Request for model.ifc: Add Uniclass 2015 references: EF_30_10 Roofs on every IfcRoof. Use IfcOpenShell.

First a look at what the model holds.

```python
import ifcopenshell

model = ifcopenshell.open("model.ifc")
print(model.schema)
print("classifications:", [c.Name for c in model.by_type("IfcClassification")])
for ifc_class in ("IfcDoor", "IfcRoof", "IfcStair", "IfcWall", "IfcWindow"):
    print(ifc_class, len(model.by_type(ifc_class)))
```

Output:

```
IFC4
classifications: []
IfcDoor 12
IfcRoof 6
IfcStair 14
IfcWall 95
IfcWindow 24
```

```python
import ifcopenshell
import ifcopenshell.api.classification

model = ifcopenshell.open("model.ifc")

system = ifcopenshell.api.classification.add_classification(model, classification="Uniclass 2015")

codes = {
    "IfcRoof": ("EF_30_10", "Roofs"),
}
for ifc_class, (code, name) in codes.items():
    products = model.by_type(ifc_class)
    ifcopenshell.api.classification.add_reference(
        model, products=products, classification=system, identification=code, name=name
    )
    print(code, len(products))

model.write("model-out.ifc")
```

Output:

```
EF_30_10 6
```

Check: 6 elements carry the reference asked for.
